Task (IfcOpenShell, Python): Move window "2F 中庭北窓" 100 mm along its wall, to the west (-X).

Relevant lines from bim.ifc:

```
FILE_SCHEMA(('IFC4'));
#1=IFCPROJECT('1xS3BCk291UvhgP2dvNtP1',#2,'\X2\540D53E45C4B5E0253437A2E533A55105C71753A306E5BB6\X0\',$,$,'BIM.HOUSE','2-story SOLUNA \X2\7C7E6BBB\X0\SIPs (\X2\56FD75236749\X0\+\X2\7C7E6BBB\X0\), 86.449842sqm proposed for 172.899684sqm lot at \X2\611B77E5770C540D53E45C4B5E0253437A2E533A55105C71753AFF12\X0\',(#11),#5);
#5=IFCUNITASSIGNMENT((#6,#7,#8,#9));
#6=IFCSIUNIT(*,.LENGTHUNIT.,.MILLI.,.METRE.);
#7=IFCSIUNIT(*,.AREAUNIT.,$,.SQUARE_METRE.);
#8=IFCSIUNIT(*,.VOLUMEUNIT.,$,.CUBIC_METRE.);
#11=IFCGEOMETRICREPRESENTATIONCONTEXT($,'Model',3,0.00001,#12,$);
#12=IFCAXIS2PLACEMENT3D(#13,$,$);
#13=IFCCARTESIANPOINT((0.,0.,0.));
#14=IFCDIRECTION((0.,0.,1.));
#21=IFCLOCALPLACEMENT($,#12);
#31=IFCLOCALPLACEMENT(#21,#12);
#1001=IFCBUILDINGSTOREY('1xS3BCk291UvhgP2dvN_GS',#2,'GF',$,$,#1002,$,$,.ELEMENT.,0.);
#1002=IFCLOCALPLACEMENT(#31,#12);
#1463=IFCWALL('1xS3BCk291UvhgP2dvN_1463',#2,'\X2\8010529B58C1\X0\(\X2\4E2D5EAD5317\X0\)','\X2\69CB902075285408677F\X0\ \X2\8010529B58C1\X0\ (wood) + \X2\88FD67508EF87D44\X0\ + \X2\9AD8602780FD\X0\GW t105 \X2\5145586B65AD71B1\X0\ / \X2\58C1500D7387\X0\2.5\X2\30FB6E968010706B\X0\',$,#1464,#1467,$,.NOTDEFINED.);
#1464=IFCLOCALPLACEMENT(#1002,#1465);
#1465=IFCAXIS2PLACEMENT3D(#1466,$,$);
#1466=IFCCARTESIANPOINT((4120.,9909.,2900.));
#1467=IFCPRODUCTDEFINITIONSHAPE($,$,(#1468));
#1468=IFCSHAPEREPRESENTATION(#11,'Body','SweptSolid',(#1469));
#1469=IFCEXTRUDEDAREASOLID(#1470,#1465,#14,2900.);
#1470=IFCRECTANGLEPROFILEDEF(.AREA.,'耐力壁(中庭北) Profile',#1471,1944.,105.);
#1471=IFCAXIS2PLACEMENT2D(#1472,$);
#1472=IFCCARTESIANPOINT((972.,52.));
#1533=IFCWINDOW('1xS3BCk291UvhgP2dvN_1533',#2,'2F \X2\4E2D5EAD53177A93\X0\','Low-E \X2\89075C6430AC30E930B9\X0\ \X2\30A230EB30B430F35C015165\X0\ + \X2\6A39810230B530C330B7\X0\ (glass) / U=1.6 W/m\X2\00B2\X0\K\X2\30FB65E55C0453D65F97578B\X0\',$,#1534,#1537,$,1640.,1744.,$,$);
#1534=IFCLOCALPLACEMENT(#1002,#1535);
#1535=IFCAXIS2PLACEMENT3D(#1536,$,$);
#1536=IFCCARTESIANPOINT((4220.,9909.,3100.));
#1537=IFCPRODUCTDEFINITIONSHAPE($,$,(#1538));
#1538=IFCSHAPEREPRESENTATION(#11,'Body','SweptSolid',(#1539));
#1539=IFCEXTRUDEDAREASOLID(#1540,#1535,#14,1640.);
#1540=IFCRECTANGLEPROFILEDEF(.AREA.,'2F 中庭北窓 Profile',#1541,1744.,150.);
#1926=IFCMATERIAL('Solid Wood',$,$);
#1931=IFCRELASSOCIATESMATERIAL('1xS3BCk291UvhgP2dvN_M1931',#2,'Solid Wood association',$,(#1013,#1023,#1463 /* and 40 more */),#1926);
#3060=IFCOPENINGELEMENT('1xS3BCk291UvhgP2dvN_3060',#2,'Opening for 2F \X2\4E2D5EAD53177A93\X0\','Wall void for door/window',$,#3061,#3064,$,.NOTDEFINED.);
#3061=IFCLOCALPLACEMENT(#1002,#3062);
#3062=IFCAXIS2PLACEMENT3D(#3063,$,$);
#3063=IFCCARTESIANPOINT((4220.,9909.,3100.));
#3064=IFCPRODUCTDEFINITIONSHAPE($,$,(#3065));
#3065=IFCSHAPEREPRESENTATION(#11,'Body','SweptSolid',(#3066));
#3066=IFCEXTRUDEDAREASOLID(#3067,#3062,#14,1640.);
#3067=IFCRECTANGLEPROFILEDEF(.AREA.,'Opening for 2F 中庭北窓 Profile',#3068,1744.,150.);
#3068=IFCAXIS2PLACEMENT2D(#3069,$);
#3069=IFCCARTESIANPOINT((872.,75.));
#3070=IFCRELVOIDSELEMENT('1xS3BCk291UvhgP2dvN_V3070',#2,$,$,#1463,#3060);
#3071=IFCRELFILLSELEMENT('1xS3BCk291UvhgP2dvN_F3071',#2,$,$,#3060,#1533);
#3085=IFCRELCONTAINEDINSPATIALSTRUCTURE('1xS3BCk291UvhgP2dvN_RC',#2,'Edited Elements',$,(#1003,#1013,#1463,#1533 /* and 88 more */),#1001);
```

```python
import ifcopenshell
import ifcopenshell.api.geometry
import ifcopenshell.util.placement

model = ifcopenshell.open("bim.ifc")

window = model.by_guid("1xS3BCk291UvhgP2dvN_1533")
opening = window.FillsVoids[0].RelatingOpeningElement
wall = opening.VoidsElements[0].RelatingBuildingElement

wall_matrix = ifcopenshell.util.placement.get_local_placement(wall.ObjectPlacement)
shift = wall_matrix[:3, 0] * -100.0
before = ifcopenshell.util.placement.get_local_placement(window.ObjectPlacement)[:3, 3].copy()

# The window is not placed relative to its opening, so move both.
for product in (opening, window):
    matrix = ifcopenshell.util.placement.get_local_placement(product.ObjectPlacement)
    matrix[:3, 3] += shift
    ifcopenshell.api.geometry.edit_object_placement(model, product=product, matrix=matrix, is_si=False)

after = ifcopenshell.util.placement.get_local_placement(window.ObjectPlacement)[:3, 3]
print("window moved by", (after - before).round(3) + 0.0)

model.write("bim-out.ifc")
```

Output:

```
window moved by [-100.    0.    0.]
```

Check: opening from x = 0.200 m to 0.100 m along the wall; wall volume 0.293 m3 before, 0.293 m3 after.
